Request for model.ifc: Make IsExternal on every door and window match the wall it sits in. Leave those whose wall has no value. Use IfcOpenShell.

First a look at what the model holds.

```python
import ifcopenshell
import ifcopenshell.util.element

model = ifcopenshell.open("model.ifc")
print(model.schema)
seen = {}
for e in model.by_type("IfcDoor") + model.by_type("IfcWindow"):
    if not e.FillsVoids:
        continue
    host = e.FillsVoids[0].RelatingOpeningElement.VoidsElements[0].RelatingBuildingElement
    own = ifcopenshell.util.element.get_pset(e, f"Pset_{e.is_a()[3:].removesuffix('StandardCase')}Common", "IsExternal")
    wall = ifcopenshell.util.element.get_pset(host, "Pset_WallCommon", "IsExternal")
    seen[e.is_a(), own, wall] = seen.get((e.is_a(), own, wall), 0) + 1
for (cls, own, wall), count in sorted(seen.items(), key=str):
    print(count, cls, "IsExternal:", own, "| host wall:", wall)
```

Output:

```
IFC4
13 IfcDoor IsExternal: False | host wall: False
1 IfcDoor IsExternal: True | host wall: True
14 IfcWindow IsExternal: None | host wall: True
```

```python
import ifcopenshell
import ifcopenshell.api.pset
import ifcopenshell.util.element

model = ifcopenshell.open("model.ifc")

count = 0
for ifc_class, pset_name in (("IfcDoor", "Pset_DoorCommon"), ("IfcWindow", "Pset_WindowCommon")):
    for e in model.by_type(ifc_class):
        if not e.FillsVoids:
            continue
        host = e.FillsVoids[0].RelatingOpeningElement.VoidsElements[0].RelatingBuildingElement
        external = ifcopenshell.util.element.get_pset(host, "Pset_WallCommon", "IsExternal")
        if external is None or ifcopenshell.util.element.get_pset(e, pset_name, "IsExternal") == external:
            continue
        pset = ifcopenshell.api.pset.add_pset(model, product=e, name=pset_name)
        ifcopenshell.api.pset.edit_pset(model, pset=pset, properties={"IsExternal": external})
        count += 1

print(count, "updated")

model.write("model_rev.ifc")
```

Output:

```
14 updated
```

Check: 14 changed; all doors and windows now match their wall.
